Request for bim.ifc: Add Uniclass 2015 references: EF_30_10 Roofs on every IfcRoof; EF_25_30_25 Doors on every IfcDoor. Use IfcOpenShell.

First a look at what the model holds.

```python
import ifcopenshell

model = ifcopenshell.open("bim.ifc")
print(model.schema)
print("classifications:", [c.Name for c in model.by_type("IfcClassification")])
for ifc_class in ("IfcDoor", "IfcRoof", "IfcStair", "IfcWall", "IfcWindow"):
    print(ifc_class, len(model.by_type(ifc_class)))
```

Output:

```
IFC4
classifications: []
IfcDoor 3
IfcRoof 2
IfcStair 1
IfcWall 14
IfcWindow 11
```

```python
import ifcopenshell
import ifcopenshell.api.classification

model = ifcopenshell.open("bim.ifc")

system = ifcopenshell.api.classification.add_classification(model, classification="Uniclass 2015")

codes = {
    "IfcRoof": ("EF_30_10", "Roofs"),
    "IfcDoor": ("EF_25_30_25", "Doors"),
}
for ifc_class, (code, name) in codes.items():
    products = model.by_type(ifc_class)
    ifcopenshell.api.classification.add_reference(
        model, products=products, classification=system, identification=code, name=name
    )
    print(code, len(products))

model.write("bim_rev.ifc")
```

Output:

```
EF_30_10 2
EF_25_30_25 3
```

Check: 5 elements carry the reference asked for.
